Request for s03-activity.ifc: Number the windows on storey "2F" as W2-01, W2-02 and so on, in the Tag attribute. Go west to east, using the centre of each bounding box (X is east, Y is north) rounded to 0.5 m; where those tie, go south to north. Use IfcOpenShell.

First a look at what the model holds.

```python
import ifcopenshell
import ifcopenshell.util.element
import ifcopenshell.util.placement

model = ifcopenshell.open("s03-activity.ifc")
print(model.schema)
storey = next(s for s in model.by_type("IfcBuildingStorey") if s.Name == "2F")
windows = [e for e in ifcopenshell.util.element.get_decomposition(storey) if e.is_a("IfcWindow")]
for e in sorted(windows, key=lambda e: e.id()):
    origin = ifcopenshell.util.placement.get_local_placement(e.ObjectPlacement)[:3, 3]
    print(e.id(), e.Tag, e.Name, origin.round(2) + 0.0, sep=" | ")
```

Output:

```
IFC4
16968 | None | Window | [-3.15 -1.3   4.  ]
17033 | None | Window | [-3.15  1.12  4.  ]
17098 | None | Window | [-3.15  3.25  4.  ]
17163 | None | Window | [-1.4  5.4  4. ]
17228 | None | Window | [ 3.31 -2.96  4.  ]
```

```python
import ifcopenshell
import ifcopenshell.geom
import ifcopenshell.util.element
import ifcopenshell.util.shape

model = ifcopenshell.open("s03-activity.ifc")
settings = ifcopenshell.geom.settings()
settings.set("use-world-coords", True)


def centre(element):
    shape = ifcopenshell.geom.create_shape(settings, element)
    return ifcopenshell.util.shape.get_bbox_centroid(shape.geometry)


storey = next(s for s in model.by_type("IfcBuildingStorey") if s.Name == "2F")
windows = [e for e in ifcopenshell.util.element.get_decomposition(storey) if e.is_a("IfcWindow")]

# Insertion points can sit at a corner or the storey origin, so sort by the geometry (in metres).
centres = {e: centre(e) for e in windows}
windows.sort(key=lambda e: (round(centres[e][0] / 0.5), centres[e][1]))

for i, e in enumerate(windows, start=1):
    number = f"W2-{i:02d}"
    e.Tag = number
    print(e.id(), number)

model.write("s03-activity_v2.ifc")
```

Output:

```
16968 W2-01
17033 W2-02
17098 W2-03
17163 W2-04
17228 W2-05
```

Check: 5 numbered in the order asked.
